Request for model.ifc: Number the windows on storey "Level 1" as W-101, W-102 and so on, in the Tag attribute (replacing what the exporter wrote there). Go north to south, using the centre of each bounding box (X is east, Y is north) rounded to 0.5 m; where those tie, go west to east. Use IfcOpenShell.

First a look at what the model holds.

```python
import ifcopenshell
import ifcopenshell.util.element
import ifcopenshell.util.placement

model = ifcopenshell.open("model.ifc")
print(model.schema)
storey = next(s for s in model.by_type("IfcBuildingStorey") if s.Name == "Level 1")
windows = [e for e in ifcopenshell.util.element.get_decomposition(storey) if e.is_a("IfcWindow")]
for e in sorted(windows, key=lambda e: e.id()):
    origin = ifcopenshell.util.placement.get_local_placement(e.ObjectPlacement)[:3, 3]
    print(e.id(), e.Tag, e.Name, origin.round(2) + 0.0, sep=" | ")
```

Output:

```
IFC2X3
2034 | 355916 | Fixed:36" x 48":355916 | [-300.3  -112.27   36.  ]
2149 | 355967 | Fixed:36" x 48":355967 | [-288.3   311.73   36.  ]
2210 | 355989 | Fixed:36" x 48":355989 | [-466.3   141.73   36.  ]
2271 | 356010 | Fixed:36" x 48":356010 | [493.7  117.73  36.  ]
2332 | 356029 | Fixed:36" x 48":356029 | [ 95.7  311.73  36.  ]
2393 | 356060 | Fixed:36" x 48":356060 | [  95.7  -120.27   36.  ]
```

```python
import ifcopenshell
import ifcopenshell.geom
import ifcopenshell.util.element
import ifcopenshell.util.shape

model = ifcopenshell.open("model.ifc")
settings = ifcopenshell.geom.settings()
settings.set("use-world-coords", True)


def centre(element):
    shape = ifcopenshell.geom.create_shape(settings, element)
    return ifcopenshell.util.shape.get_bbox_centroid(shape.geometry)


storey = next(s for s in model.by_type("IfcBuildingStorey") if s.Name == "Level 1")
windows = [e for e in ifcopenshell.util.element.get_decomposition(storey) if e.is_a("IfcWindow")]

# Insertion points can sit at a corner or the storey origin, so sort by the geometry (in metres).
centres = {e: centre(e) for e in windows}
windows.sort(key=lambda e: (-round(centres[e][1] / 0.5), centres[e][0]))

for i, e in enumerate(windows, start=1):
    number = f"W-1{i:02d}"
    e.Tag = number
    print(e.id(), number)

model.write("model_v2.ifc")
```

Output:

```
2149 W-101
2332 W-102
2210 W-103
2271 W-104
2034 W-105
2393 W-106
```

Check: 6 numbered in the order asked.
